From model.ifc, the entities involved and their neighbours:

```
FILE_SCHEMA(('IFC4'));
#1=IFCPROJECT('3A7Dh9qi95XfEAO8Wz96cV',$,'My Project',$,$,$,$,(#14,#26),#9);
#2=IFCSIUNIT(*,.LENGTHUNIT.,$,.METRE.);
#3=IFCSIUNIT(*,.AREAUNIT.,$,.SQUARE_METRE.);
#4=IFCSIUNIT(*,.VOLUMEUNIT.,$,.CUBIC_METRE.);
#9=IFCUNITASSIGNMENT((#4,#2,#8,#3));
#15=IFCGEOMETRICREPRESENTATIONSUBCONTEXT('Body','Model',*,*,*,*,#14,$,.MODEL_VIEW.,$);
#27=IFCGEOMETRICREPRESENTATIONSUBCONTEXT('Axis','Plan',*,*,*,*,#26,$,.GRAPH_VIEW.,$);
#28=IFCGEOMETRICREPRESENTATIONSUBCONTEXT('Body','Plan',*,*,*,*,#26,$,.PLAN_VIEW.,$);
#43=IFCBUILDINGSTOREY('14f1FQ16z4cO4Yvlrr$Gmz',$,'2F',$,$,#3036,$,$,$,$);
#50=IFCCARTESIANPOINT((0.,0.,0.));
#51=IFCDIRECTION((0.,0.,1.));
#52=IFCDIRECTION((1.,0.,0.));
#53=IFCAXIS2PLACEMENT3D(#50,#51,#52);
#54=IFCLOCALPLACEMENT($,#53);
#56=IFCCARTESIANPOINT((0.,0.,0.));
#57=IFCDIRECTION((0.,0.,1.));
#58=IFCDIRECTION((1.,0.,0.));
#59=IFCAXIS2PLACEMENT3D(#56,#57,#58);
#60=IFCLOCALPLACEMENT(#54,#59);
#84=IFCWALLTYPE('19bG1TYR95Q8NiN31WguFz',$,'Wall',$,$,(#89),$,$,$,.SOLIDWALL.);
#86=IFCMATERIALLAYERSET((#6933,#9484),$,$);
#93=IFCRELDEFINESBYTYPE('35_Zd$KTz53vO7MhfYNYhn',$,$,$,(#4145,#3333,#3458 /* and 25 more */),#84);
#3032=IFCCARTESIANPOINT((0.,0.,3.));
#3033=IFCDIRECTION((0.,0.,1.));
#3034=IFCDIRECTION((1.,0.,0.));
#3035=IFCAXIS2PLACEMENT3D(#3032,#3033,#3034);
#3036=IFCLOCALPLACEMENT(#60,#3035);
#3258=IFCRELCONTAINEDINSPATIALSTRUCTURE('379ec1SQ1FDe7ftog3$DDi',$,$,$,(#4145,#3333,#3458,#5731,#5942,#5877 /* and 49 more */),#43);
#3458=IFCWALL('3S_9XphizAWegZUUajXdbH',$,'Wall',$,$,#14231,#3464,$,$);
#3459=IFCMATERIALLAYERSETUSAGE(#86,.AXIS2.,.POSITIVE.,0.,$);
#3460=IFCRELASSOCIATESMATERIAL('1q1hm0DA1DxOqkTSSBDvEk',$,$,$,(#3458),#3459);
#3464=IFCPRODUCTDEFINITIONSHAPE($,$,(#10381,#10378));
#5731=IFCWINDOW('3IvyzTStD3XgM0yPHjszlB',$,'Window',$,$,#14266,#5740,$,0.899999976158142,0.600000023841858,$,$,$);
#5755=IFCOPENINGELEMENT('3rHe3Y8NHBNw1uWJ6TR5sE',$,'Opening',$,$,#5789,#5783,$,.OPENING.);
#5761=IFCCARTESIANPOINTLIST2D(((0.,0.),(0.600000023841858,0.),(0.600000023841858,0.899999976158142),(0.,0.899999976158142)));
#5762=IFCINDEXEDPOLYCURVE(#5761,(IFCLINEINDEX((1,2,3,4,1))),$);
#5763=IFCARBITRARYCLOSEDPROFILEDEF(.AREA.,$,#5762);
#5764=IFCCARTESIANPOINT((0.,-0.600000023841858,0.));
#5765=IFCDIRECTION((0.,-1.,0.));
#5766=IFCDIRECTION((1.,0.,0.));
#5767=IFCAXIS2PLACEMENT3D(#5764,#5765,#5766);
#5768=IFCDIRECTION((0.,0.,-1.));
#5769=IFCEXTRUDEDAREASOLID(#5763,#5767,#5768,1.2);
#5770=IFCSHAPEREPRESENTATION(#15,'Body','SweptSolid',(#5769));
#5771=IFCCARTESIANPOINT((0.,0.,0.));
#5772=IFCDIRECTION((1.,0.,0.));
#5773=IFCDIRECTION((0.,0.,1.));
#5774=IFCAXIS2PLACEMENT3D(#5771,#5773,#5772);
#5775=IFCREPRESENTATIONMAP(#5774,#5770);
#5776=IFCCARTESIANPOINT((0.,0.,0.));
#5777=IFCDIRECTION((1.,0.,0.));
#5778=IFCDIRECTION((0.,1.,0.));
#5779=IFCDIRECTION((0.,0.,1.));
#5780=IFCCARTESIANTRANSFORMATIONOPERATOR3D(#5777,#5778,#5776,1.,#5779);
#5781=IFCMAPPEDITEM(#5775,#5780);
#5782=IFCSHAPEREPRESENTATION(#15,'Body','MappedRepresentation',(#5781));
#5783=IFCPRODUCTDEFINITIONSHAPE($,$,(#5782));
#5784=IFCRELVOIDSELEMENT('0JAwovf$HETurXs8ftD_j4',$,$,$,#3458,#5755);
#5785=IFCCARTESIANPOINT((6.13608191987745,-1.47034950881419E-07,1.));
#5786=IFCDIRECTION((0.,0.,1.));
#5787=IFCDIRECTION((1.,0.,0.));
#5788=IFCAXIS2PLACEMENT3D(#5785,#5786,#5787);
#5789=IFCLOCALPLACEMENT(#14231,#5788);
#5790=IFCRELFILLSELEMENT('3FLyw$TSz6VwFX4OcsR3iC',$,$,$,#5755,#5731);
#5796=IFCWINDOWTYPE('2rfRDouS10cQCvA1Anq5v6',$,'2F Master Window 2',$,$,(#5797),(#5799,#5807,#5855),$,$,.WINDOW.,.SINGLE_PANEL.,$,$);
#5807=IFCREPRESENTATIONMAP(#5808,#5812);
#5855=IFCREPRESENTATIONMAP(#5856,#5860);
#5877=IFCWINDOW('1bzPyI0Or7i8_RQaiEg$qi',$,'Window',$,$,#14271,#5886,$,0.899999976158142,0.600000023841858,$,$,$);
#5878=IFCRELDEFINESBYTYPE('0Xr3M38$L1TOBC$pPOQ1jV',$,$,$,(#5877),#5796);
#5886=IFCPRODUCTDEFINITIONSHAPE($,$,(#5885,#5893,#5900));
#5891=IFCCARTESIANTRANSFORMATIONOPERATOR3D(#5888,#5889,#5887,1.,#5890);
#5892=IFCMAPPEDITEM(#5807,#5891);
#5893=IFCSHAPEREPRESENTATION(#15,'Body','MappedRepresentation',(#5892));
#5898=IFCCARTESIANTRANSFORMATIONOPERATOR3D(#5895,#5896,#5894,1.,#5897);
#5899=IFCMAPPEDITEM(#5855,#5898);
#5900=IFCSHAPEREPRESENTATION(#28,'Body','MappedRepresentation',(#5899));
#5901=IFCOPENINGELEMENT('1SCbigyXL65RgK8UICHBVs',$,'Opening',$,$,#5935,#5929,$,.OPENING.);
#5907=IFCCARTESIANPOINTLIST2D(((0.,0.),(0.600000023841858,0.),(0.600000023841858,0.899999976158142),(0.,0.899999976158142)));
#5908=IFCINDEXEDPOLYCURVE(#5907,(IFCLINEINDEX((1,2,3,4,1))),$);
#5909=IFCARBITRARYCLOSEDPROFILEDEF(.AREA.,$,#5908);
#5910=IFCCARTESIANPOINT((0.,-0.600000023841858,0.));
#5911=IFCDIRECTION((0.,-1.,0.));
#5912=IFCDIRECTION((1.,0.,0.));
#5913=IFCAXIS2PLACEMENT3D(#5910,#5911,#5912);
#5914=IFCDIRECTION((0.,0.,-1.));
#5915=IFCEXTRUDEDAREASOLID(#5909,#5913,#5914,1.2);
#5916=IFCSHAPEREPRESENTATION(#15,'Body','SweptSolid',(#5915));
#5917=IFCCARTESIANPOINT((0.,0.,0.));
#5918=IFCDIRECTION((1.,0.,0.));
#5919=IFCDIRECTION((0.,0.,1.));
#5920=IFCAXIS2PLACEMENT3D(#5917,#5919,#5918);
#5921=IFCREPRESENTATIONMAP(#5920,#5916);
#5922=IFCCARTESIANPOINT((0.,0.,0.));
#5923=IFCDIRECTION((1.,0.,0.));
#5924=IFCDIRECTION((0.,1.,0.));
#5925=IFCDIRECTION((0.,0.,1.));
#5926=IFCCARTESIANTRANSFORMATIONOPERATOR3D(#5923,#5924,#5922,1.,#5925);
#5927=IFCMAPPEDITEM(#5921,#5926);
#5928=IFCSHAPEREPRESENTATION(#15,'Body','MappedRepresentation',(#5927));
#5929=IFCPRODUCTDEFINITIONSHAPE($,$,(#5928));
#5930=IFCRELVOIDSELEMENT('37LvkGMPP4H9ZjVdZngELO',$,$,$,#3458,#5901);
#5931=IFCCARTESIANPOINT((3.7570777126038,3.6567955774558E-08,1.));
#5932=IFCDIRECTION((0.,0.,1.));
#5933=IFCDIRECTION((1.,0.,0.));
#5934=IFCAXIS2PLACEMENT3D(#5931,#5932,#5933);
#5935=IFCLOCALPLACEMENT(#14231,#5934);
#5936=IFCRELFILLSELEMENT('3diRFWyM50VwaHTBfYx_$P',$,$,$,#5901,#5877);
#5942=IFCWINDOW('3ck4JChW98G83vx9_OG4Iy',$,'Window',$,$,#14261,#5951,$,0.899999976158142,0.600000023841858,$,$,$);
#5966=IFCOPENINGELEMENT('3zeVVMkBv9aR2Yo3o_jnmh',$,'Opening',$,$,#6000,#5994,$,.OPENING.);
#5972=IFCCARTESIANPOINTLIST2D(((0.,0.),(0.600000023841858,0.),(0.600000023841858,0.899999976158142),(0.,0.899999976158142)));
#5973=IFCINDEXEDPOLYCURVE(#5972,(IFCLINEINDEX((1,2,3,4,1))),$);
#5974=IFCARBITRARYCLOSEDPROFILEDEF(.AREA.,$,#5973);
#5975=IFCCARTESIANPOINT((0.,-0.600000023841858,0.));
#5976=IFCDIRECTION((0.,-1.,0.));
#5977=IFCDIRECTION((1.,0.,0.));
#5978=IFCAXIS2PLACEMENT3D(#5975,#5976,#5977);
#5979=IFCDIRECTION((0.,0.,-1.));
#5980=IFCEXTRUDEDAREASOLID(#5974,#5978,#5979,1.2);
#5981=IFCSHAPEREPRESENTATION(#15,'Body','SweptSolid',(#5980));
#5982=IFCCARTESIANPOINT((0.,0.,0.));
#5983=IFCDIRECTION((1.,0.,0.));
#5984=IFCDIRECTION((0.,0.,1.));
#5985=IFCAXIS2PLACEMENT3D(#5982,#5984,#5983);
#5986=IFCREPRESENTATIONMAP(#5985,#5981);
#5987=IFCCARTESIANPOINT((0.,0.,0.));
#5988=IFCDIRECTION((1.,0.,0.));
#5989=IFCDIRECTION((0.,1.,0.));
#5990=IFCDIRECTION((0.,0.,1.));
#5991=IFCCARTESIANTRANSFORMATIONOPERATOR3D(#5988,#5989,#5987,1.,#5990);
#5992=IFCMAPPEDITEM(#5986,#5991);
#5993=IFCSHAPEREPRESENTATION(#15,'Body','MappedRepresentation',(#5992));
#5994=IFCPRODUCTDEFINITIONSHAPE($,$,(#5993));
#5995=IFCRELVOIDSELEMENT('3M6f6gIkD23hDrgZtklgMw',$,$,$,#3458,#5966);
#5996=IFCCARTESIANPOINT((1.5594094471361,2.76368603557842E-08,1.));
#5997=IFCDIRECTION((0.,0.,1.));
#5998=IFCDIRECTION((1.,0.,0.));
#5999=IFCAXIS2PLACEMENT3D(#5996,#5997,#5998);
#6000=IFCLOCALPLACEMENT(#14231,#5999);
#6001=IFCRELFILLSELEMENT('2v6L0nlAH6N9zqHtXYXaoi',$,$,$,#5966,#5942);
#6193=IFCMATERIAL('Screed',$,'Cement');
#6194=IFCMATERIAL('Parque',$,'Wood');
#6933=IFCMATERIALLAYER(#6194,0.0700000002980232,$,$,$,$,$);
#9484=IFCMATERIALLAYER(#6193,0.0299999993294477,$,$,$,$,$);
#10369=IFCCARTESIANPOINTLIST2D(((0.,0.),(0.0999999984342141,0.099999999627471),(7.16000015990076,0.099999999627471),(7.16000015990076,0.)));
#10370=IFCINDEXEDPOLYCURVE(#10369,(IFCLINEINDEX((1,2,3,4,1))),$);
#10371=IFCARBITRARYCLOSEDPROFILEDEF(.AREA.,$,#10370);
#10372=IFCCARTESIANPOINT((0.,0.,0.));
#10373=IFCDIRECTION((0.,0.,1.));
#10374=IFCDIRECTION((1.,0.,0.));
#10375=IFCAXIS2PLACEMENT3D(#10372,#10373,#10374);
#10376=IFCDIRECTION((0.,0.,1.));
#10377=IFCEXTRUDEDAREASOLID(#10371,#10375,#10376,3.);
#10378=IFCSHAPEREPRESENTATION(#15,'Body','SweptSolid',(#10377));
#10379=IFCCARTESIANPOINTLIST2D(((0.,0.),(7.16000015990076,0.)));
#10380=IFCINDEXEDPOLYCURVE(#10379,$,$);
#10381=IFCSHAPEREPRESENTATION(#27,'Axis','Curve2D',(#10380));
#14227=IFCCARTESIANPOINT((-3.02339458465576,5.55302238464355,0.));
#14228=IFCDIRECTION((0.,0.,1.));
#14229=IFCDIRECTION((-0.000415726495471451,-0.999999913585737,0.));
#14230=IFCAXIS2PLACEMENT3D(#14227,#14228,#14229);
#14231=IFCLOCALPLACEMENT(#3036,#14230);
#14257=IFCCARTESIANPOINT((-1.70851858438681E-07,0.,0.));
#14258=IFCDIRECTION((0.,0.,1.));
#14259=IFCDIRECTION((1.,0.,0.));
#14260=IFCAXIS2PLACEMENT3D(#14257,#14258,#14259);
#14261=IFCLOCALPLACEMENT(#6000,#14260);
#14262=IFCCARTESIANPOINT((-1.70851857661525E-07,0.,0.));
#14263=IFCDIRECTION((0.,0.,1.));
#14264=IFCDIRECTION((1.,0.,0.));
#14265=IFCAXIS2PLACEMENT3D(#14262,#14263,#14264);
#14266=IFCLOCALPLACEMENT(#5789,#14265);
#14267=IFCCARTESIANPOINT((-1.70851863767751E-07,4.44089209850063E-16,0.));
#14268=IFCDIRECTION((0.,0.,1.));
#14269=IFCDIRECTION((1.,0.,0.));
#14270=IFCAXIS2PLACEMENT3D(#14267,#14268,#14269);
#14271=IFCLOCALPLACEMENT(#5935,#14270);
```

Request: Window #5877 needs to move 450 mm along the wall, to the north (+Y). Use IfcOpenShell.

```python
import ifcopenshell
import ifcopenshell.api.geometry
import ifcopenshell.util.placement
import ifcopenshell.util.unit

model = ifcopenshell.open("model.ifc")
unit_scale = ifcopenshell.util.unit.calculate_unit_scale(model)

window = model.by_id(5877)
opening = window.FillsVoids[0].RelatingOpeningElement
wall = opening.VoidsElements[0].RelatingBuildingElement

wall_matrix = ifcopenshell.util.placement.get_local_placement(wall.ObjectPlacement)
shift = wall_matrix[:3, 0] * -0.45 / unit_scale
before = ifcopenshell.util.placement.get_local_placement(window.ObjectPlacement)[:3, 3].copy()

# The window is placed relative to its opening, so it follows when the opening moves.
matrix = ifcopenshell.util.placement.get_local_placement(opening.ObjectPlacement)
matrix[:3, 3] += shift
ifcopenshell.api.geometry.edit_object_placement(
    model, product=opening, matrix=matrix, is_si=False, should_transform_children=True
)

after = ifcopenshell.util.placement.get_local_placement(window.ObjectPlacement)[:3, 3]
print("window moved by", (after - before).round(3) + 0.0)

model.write("model-out.ifc")
```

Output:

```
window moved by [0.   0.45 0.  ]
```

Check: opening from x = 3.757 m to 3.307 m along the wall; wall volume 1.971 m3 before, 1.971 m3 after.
